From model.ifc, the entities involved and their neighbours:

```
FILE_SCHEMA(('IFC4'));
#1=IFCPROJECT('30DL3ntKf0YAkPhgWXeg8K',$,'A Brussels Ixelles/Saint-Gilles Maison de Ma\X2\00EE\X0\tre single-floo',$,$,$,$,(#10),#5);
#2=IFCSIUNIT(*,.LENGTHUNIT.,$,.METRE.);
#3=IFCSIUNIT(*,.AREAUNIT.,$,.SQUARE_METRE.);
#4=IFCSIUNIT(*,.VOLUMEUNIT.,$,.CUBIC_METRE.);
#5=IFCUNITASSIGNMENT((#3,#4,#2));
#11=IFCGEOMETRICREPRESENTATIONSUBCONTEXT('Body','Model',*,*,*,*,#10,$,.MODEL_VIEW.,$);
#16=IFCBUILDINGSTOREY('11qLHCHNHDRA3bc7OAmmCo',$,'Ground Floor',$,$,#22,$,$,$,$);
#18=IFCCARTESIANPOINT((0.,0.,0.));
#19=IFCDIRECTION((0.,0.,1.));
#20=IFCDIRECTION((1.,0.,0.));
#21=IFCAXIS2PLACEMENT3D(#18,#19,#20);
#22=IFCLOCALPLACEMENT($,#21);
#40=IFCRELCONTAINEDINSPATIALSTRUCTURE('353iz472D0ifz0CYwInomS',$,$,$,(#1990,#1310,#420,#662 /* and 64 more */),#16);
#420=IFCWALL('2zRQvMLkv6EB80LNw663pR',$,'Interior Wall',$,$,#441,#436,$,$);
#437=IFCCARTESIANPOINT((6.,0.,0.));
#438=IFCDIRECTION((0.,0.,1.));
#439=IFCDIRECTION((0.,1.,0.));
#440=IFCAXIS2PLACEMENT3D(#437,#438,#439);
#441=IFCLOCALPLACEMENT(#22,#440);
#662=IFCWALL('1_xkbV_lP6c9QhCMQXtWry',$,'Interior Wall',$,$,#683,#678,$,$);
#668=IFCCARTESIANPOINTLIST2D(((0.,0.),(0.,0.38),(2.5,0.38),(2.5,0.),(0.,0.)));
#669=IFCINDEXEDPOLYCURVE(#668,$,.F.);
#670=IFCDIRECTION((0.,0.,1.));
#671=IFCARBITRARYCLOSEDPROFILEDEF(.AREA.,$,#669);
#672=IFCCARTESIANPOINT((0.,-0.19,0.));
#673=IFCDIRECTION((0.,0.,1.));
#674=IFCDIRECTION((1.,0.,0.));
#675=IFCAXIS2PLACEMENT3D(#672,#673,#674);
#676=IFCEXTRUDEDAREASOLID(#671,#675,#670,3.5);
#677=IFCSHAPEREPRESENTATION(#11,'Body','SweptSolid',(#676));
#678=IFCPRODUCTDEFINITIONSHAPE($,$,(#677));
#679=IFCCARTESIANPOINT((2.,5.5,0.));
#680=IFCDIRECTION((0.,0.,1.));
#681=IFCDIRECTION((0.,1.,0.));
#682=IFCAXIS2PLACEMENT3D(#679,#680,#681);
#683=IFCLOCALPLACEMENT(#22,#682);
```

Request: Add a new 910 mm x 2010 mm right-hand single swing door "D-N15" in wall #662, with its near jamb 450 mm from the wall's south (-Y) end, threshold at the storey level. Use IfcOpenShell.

```python
import numpy as np
import ifcopenshell
import ifcopenshell.api.feature
import ifcopenshell.api.geometry
import ifcopenshell.api.root
import ifcopenshell.api.spatial
import ifcopenshell.geom
import ifcopenshell.util.element
import ifcopenshell.util.placement
import ifcopenshell.util.representation
import ifcopenshell.util.shape
import ifcopenshell.util.unit

model = ifcopenshell.open("model.ifc")
unit_scale = ifcopenshell.util.unit.calculate_unit_scale(model)
settings = ifcopenshell.geom.settings()


def volume(element):
    """Net volume in cubic metres, openings subtracted."""
    shape = ifcopenshell.geom.create_shape(settings, element)
    return ifcopenshell.util.shape.get_volume(shape.geometry)


wall = model.by_guid("1_xkbV_lP6c9QhCMQXtWry")
storey = ifcopenshell.util.element.get_container(wall, ifc_class="IfcBuildingStorey")
context = ifcopenshell.util.representation.get_context(model, "Model", "Body", "MODEL_VIEW")
before = volume(wall)

width, height, from_end, sill = 0.91, 2.01, 0.45, 0.0  # metres

# The wall runs along its own X axis, and the end named is its -X end.
wall_shape = ifcopenshell.geom.create_shape(settings, wall)
x, y, z = ifcopenshell.util.shape.get_vertices(wall_shape.geometry).T
start = x.min() + from_end
face, thickness = float(y.min()), float(y.max() - y.min())
wall_matrix = ifcopenshell.util.placement.get_local_placement(wall.ObjectPlacement)
level = ifcopenshell.util.placement.get_local_placement(storey.ObjectPlacement)[2, 3]


def in_wall(x, y):
    """Placement at x, y metres in the wall's axes, at sill height."""
    matrix = wall_matrix.copy()
    matrix[:, 3] = wall_matrix @ np.array([x / unit_scale, y / unit_scale, 0.0, 1.0])
    matrix[2, 3] = level + sill / unit_scale
    return matrix


# Opening: a box that overshoots both wall faces by 50 mm.
opening = ifcopenshell.api.root.create_entity(model, ifc_class="IfcOpeningElement", predefined_type="OPENING")
box = ifcopenshell.api.geometry.add_wall_representation(
    model, context=context, length=width, height=height, thickness=thickness + 0.1
)
ifcopenshell.api.geometry.assign_representation(model, product=opening, representation=box)
ifcopenshell.api.geometry.edit_object_placement(model, product=opening, matrix=in_wall(start, face - 0.05), is_si=False)
ifcopenshell.api.feature.add_feature(model, feature=opening, element=wall)

door = ifcopenshell.api.root.create_entity(model, ifc_class="IfcDoor", name="D-N15", predefined_type="DOOR")
door.OverallWidth, door.OverallHeight = width / unit_scale, height / unit_scale
door.OperationType = "SINGLE_SWING_RIGHT"
body = ifcopenshell.api.geometry.add_door_representation(
    model,
    context=context,
    overall_width=door.OverallWidth,
    overall_height=door.OverallHeight,
    operation_type="SINGLE_SWING_RIGHT",
    lining_properties={"LiningDepth": thickness / unit_scale, "ThresholdDepth": thickness / unit_scale},
)
ifcopenshell.api.geometry.assign_representation(model, product=door, representation=body)
ifcopenshell.api.spatial.assign_container(model, products=[door], relating_structure=storey)
ifcopenshell.api.feature.add_filling(model, opening=opening, element=door)

# The lining spans the wall, so the door starts at the wall face.
ifcopenshell.api.geometry.edit_object_placement(model, product=door, matrix=in_wall(start, face), is_si=False)

after = volume(wall)

print(f"wall volume {before:.3f} -> {after:.3f} m3")

model.write("model-out.ifc")
```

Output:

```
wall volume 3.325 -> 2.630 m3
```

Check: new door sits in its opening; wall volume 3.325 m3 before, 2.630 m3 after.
